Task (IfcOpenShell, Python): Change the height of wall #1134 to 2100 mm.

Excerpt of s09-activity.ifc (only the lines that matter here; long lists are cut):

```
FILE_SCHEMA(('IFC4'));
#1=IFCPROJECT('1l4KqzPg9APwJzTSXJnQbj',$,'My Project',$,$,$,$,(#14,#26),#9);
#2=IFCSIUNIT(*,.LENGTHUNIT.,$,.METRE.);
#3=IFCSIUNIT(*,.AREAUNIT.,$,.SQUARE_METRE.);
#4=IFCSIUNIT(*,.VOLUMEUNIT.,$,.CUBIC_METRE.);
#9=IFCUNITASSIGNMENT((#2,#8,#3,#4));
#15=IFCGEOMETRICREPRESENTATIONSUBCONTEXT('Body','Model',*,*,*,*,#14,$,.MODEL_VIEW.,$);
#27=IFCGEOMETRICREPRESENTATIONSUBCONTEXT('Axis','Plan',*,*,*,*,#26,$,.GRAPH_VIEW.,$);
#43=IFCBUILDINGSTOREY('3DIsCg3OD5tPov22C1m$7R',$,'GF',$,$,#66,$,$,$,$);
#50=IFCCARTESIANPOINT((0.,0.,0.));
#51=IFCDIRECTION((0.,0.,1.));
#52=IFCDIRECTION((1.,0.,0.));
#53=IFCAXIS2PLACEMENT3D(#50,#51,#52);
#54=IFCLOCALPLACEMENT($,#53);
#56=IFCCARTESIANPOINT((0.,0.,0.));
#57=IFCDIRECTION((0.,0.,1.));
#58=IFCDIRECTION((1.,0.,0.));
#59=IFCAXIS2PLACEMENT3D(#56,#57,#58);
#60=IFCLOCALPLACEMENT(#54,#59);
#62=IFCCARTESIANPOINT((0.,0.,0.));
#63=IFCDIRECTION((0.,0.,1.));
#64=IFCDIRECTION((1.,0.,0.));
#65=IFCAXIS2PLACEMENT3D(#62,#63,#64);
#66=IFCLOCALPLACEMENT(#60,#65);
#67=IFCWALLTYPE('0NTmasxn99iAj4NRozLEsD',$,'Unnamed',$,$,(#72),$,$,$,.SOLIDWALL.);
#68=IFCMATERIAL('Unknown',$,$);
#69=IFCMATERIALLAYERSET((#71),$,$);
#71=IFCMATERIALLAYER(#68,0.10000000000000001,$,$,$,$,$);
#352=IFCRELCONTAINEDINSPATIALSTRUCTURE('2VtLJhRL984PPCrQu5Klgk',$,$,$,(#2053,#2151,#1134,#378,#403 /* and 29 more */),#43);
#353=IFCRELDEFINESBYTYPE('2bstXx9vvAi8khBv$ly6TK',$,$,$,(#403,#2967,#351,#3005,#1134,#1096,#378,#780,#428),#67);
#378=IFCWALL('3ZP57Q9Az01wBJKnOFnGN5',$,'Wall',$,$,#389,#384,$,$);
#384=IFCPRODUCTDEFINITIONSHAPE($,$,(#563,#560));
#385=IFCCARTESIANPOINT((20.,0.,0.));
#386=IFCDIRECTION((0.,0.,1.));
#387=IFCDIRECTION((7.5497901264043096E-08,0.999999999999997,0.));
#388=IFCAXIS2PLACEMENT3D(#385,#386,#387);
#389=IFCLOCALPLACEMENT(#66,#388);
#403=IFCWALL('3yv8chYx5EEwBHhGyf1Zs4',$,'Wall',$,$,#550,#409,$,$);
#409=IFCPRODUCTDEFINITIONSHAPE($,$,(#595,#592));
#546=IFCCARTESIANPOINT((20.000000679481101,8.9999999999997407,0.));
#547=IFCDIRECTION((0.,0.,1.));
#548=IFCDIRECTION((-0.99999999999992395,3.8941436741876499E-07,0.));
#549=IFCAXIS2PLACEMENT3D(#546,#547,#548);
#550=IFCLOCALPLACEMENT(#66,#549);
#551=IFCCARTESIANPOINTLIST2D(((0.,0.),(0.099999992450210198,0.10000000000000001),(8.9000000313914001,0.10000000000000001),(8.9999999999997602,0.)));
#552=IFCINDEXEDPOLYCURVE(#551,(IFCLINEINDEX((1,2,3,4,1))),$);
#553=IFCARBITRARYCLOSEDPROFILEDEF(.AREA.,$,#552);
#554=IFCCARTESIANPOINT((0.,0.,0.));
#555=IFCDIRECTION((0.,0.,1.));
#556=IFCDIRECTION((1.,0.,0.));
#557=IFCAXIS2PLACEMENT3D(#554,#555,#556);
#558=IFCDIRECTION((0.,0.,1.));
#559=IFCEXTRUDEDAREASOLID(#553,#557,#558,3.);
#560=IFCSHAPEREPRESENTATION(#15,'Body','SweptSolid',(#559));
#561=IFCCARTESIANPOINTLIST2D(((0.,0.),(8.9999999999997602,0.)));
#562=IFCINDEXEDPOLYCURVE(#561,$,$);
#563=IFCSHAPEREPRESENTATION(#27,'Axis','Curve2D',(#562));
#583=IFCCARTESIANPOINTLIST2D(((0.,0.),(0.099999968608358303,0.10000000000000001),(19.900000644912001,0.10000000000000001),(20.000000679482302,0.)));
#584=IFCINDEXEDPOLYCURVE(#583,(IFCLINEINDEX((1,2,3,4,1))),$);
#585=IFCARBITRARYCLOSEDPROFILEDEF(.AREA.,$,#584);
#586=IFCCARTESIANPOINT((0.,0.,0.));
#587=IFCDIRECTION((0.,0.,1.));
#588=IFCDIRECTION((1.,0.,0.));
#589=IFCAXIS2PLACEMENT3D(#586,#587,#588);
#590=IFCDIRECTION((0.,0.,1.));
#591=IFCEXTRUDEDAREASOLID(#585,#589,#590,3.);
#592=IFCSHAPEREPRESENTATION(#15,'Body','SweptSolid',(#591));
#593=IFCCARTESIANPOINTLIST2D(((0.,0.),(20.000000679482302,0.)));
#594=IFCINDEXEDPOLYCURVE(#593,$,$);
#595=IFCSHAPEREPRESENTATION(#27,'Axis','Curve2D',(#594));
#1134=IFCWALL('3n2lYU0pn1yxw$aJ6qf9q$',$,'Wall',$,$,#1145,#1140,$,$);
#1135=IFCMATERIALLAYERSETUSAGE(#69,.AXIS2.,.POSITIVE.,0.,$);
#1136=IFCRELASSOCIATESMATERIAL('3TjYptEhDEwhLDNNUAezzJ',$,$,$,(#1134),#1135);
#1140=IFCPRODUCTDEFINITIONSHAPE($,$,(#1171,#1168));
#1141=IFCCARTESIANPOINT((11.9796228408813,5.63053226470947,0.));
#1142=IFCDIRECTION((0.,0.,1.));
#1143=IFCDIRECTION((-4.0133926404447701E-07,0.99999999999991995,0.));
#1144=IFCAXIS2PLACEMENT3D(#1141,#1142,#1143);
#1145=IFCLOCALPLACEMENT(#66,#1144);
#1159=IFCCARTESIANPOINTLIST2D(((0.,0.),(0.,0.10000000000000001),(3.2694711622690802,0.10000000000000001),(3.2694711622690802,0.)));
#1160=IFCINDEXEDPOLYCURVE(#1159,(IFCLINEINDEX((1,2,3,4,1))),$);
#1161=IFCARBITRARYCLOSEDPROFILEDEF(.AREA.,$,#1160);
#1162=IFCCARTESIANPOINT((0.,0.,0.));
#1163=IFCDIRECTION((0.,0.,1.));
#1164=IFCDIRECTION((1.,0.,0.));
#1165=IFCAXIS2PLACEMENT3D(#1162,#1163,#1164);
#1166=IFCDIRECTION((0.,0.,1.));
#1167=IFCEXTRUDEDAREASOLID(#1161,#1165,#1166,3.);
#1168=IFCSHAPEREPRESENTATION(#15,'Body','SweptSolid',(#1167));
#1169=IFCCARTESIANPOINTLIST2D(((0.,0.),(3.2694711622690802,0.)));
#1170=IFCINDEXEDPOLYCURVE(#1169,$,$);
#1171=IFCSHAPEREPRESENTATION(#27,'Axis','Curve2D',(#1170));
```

```python
import ifcopenshell
import ifcopenshell.geom
import ifcopenshell.util.representation
import ifcopenshell.util.shape

model = ifcopenshell.open("s09-activity.ifc")
settings = ifcopenshell.geom.settings()


def volume(element):
    """Net volume in cubic metres, openings subtracted."""
    shape = ifcopenshell.geom.create_shape(settings, element)
    return ifcopenshell.util.shape.get_volume(shape.geometry)


wall = model.by_id(1134)
before = volume(wall)

body = ifcopenshell.util.representation.get_representation(wall, "Model", "Body")
solid = body.Items[0]
old_height = solid.Depth
solid.Depth = 2.1
after = volume(wall)

print(f"height {old_height:g} -> {solid.Depth:g}, volume {before:.3f} -> {after:.3f} m3")

model.write("s09-activity-out.ifc")
```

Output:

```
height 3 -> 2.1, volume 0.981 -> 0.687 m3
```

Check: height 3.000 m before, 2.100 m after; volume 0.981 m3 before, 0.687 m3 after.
